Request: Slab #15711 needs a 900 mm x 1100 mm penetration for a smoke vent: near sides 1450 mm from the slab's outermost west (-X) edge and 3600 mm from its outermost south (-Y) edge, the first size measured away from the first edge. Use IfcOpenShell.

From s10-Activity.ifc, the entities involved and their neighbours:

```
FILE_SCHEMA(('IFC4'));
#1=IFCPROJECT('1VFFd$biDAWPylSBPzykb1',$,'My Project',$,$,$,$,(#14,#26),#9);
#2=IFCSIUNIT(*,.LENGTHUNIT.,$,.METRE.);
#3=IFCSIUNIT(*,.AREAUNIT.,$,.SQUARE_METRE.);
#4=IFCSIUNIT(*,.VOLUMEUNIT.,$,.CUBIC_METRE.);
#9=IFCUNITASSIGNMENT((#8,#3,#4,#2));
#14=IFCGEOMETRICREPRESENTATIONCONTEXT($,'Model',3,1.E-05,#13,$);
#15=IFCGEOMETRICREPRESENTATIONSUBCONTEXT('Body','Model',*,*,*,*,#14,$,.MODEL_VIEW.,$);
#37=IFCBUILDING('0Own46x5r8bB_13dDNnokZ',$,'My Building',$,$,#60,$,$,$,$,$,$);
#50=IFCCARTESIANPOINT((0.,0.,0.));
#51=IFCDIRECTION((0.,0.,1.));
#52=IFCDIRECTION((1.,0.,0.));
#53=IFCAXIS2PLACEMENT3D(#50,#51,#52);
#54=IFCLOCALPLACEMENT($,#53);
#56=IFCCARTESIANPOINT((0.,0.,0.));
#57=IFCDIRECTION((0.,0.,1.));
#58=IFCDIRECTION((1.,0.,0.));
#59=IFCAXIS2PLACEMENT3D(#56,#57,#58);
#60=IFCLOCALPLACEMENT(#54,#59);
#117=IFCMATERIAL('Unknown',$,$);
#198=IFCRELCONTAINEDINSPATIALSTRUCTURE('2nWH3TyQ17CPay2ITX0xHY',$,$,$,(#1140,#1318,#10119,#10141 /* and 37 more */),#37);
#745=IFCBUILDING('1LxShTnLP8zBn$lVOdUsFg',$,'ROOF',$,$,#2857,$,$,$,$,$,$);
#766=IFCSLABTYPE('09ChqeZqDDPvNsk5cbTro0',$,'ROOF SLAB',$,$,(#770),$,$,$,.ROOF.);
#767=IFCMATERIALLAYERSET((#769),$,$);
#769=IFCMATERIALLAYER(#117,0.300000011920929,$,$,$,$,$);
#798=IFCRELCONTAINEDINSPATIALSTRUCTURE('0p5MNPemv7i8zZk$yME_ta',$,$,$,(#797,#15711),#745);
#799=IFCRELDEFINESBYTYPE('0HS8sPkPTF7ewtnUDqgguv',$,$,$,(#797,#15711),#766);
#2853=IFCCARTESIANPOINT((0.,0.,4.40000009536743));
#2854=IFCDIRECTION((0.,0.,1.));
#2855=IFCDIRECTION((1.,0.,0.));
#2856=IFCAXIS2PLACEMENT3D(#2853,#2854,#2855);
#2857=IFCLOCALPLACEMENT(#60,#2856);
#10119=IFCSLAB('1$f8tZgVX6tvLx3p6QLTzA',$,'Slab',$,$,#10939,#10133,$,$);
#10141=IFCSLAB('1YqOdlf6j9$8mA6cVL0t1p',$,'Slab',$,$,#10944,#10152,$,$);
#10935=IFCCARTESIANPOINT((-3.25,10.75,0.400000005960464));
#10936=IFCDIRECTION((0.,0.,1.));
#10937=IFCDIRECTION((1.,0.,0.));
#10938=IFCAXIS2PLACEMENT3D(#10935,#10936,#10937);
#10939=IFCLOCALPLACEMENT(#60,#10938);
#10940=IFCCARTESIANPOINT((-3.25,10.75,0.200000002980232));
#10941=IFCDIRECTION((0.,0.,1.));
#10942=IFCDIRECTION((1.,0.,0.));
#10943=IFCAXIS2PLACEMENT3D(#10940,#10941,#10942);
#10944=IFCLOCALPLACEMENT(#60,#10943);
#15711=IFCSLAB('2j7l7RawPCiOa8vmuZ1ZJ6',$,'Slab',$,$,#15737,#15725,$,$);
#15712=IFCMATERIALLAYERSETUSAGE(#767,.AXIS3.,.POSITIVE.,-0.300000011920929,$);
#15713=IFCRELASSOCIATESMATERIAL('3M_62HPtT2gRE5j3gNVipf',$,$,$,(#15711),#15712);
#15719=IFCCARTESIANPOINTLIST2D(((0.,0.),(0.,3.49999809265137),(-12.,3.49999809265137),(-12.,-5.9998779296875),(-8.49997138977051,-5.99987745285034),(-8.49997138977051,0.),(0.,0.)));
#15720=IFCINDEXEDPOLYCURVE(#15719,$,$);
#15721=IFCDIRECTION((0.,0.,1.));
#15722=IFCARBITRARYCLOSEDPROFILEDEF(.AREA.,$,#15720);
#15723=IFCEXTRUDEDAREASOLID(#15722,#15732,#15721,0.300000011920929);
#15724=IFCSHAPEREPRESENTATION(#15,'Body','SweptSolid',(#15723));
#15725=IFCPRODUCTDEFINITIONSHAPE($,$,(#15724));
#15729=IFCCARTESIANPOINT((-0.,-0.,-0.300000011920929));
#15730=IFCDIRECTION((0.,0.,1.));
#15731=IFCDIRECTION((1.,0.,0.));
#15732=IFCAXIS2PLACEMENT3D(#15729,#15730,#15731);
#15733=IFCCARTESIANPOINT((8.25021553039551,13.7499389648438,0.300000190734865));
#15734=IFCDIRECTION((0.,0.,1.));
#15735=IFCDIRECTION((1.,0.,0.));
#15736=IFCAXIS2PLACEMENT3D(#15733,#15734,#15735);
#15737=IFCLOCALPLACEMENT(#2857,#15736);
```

```python
import numpy as np
import ifcopenshell
import ifcopenshell.api.feature
import ifcopenshell.api.geometry
import ifcopenshell.api.root
import ifcopenshell.geom
import ifcopenshell.util.placement
import ifcopenshell.util.representation
import ifcopenshell.util.shape
import ifcopenshell.util.unit

model = ifcopenshell.open("s10-Activity.ifc")
unit_scale = ifcopenshell.util.unit.calculate_unit_scale(model)
settings = ifcopenshell.geom.settings()


def volume(element):
    """Net volume in cubic metres, openings subtracted."""
    shape = ifcopenshell.geom.create_shape(settings, element)
    return ifcopenshell.util.shape.get_volume(shape.geometry)


slab = model.by_id(15711)
before = volume(slab)

# Extent in the slab's own axes, in metres. The edges named are its -X and -Y sides.
slab_shape = ifcopenshell.geom.create_shape(settings, slab)
vertices = ifcopenshell.util.shape.get_vertices(slab_shape.geometry)
x_min, y_min, bottom = vertices.min(axis=0)
top = vertices[:, 2].max()

opening = ifcopenshell.api.root.create_entity(model, ifc_class="IfcOpeningElement", name="Smoke vent opening", predefined_type="OPENING")
context = ifcopenshell.util.representation.get_context(model, "Model", "Body", "MODEL_VIEW")
width, depth = 0.9, 1.1
outline = [(0.0, 0.0), (width, 0.0), (width, depth), (0.0, depth), (0.0, 0.0)]
# Overshoot both faces by 50 mm so the cut is clean.
shape = ifcopenshell.api.geometry.add_slab_representation(
    model, context=context, depth=top - bottom + 0.1, polyline=outline
)
ifcopenshell.api.geometry.assign_representation(model, product=opening, representation=shape)

matrix = ifcopenshell.util.placement.get_local_placement(slab.ObjectPlacement)
matrix[:, 3] = matrix @ np.append(np.array([x_min + 1.45, y_min + 3.6, bottom - 0.05]) / unit_scale, 1.0)
ifcopenshell.api.geometry.edit_object_placement(model, product=opening, matrix=matrix, is_si=False)
ifcopenshell.api.feature.add_feature(model, feature=opening, element=slab)

after = volume(slab)

print(f"slab volume {before:.3f} -> {after:.3f} m3")

model.write("s10-Activity_v2.ifc")
```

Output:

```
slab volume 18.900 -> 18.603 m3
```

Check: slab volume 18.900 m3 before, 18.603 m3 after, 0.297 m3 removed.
